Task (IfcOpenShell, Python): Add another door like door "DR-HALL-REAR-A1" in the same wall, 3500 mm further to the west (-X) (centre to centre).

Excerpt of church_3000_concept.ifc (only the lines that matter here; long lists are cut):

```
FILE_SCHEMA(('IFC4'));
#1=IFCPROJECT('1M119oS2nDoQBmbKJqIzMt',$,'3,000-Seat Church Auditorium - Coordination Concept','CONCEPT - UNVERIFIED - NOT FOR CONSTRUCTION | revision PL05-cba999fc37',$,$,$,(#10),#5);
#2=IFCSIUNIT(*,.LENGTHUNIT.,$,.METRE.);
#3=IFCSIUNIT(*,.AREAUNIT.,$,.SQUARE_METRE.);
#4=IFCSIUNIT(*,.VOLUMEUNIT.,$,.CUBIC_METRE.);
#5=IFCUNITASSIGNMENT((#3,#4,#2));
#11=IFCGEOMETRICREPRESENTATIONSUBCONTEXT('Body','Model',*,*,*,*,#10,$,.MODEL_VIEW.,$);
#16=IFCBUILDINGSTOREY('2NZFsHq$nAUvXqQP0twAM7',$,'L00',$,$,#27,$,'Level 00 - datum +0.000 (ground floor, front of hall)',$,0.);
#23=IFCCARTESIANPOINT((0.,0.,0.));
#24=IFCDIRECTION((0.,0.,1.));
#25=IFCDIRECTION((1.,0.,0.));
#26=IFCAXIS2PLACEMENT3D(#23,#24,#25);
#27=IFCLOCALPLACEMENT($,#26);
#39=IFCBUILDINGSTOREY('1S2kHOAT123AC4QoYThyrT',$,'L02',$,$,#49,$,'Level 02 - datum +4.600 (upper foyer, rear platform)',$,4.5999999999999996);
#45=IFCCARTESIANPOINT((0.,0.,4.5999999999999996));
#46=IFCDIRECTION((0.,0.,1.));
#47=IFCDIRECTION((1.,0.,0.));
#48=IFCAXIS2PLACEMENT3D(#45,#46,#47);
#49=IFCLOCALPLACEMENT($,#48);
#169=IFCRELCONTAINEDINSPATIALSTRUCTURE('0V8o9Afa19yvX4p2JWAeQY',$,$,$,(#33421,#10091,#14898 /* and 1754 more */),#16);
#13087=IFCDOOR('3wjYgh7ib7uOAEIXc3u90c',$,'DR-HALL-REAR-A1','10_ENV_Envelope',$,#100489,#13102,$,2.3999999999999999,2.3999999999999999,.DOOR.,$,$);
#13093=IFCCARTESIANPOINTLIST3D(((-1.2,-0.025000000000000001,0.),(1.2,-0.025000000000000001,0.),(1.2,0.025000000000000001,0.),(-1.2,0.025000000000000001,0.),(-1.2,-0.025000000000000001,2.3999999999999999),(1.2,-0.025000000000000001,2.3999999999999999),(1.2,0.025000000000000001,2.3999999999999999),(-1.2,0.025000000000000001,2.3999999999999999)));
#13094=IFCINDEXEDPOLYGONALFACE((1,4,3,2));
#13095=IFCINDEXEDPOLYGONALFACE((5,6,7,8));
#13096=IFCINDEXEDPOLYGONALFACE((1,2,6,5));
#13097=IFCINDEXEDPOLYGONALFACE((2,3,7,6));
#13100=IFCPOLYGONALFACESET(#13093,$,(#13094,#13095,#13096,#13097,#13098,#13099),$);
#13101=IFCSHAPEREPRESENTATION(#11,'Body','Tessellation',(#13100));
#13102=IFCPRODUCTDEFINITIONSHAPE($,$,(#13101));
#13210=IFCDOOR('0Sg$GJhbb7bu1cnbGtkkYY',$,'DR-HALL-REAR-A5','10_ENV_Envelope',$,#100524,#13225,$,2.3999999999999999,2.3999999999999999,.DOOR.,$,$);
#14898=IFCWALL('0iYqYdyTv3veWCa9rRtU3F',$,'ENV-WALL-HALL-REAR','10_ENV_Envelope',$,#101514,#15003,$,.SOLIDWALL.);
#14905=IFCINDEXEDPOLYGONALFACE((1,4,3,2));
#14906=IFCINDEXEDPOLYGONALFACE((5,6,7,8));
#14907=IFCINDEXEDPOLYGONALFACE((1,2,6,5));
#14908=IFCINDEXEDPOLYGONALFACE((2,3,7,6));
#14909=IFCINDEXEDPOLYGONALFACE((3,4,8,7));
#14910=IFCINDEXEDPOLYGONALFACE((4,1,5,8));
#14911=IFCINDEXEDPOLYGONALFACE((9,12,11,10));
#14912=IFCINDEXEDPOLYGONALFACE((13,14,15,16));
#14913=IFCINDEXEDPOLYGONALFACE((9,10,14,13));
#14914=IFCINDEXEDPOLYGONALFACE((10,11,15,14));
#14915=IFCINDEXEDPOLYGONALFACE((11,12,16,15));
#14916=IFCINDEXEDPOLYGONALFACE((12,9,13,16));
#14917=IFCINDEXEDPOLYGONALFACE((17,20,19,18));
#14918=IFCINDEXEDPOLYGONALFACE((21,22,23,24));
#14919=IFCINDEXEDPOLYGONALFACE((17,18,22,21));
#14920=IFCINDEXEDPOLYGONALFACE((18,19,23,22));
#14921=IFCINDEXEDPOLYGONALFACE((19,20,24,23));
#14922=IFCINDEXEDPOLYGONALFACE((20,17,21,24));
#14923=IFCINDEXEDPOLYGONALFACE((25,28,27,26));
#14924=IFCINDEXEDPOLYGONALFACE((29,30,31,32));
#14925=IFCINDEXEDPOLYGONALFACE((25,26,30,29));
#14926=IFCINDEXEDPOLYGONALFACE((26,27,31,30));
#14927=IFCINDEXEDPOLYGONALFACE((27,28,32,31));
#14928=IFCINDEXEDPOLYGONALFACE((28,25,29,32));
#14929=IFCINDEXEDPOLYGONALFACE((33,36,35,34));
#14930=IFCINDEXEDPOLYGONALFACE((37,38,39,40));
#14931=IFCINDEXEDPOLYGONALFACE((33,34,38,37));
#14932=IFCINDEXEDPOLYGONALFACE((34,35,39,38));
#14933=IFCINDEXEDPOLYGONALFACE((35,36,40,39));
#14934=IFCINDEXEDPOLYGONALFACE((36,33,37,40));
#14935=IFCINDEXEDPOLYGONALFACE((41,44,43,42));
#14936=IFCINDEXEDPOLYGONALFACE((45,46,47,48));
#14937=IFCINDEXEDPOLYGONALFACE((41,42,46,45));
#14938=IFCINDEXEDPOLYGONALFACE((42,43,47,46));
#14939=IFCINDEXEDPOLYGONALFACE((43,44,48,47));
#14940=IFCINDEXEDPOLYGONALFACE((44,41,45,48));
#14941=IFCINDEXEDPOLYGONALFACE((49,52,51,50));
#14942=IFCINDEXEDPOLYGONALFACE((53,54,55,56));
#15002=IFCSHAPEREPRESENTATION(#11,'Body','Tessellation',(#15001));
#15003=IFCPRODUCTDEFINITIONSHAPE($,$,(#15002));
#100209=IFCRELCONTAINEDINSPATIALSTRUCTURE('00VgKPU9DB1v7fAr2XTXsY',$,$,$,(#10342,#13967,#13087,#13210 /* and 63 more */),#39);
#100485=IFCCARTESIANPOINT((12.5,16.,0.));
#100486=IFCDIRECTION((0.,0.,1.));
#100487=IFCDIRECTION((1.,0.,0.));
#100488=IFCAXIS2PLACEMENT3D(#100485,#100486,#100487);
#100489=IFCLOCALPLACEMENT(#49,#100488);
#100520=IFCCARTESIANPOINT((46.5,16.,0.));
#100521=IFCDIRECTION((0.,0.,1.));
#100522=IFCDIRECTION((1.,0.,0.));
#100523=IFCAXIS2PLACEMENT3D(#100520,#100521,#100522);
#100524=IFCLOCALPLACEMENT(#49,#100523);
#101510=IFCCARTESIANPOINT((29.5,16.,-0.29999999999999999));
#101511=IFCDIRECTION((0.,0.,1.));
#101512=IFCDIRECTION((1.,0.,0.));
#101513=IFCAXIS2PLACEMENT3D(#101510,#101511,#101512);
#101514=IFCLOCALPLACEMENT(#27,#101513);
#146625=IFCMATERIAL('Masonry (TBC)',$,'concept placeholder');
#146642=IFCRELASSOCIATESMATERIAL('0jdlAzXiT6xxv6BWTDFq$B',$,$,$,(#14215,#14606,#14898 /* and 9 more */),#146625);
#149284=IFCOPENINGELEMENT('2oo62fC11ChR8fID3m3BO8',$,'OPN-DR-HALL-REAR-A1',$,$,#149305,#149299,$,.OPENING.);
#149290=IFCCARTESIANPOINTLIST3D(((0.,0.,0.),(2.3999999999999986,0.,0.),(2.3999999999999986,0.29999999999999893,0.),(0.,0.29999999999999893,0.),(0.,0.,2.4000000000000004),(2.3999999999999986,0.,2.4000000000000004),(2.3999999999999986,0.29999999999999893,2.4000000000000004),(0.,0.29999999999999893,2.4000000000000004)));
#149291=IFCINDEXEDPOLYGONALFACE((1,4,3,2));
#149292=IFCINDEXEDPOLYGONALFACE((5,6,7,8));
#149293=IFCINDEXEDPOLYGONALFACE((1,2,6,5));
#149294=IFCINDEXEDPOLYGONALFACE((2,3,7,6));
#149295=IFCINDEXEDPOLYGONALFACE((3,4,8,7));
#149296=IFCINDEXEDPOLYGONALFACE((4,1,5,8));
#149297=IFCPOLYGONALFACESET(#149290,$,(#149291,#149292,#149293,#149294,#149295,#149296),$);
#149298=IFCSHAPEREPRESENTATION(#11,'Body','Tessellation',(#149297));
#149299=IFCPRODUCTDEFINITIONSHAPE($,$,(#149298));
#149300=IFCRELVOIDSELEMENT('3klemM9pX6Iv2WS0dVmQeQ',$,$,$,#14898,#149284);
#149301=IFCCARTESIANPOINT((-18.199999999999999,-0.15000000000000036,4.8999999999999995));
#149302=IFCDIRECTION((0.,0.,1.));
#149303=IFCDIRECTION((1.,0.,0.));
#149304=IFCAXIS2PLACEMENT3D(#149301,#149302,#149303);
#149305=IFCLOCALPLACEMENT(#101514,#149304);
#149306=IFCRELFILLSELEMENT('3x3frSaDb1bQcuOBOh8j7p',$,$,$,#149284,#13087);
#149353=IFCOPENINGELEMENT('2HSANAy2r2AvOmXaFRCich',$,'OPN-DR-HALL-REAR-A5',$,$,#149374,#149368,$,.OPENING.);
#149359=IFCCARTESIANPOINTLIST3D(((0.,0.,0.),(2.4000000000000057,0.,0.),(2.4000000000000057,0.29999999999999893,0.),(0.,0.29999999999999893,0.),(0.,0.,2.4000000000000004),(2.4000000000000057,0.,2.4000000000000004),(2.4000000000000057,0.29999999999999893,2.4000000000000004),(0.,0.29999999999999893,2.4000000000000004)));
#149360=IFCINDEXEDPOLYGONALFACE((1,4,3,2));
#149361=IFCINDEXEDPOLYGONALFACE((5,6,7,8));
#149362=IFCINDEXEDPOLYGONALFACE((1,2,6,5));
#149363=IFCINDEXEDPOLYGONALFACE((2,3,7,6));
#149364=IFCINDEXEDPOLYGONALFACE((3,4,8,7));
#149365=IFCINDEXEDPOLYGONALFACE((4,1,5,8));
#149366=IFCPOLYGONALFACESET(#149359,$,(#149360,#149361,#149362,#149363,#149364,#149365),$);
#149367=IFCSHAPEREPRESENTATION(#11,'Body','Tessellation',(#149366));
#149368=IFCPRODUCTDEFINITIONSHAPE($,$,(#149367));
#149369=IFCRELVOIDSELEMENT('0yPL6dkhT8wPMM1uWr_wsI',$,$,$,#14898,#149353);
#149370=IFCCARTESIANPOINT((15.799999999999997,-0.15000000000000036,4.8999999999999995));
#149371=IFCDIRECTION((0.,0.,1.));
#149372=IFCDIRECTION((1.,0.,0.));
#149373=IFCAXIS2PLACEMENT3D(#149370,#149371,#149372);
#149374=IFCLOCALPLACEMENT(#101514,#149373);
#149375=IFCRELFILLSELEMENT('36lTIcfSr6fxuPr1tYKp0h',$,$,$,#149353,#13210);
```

```python
import ifcopenshell
import ifcopenshell.api.feature
import ifcopenshell.api.geometry
import ifcopenshell.api.root
import ifcopenshell.geom
import ifcopenshell.util.element
import ifcopenshell.util.placement
import ifcopenshell.util.shape
import ifcopenshell.util.unit

model = ifcopenshell.open("church_3000_concept.ifc")
unit_scale = ifcopenshell.util.unit.calculate_unit_scale(model)
settings = ifcopenshell.geom.settings()


def volume(element):
    """Net volume in cubic metres, openings subtracted."""
    shape = ifcopenshell.geom.create_shape(settings, element)
    return ifcopenshell.util.shape.get_volume(shape.geometry)


door = model.by_id(13087)
opening = door.FillsVoids[0].RelatingOpeningElement
wall = opening.VoidsElements[0].RelatingBuildingElement
before = volume(wall)
shift = ifcopenshell.util.placement.get_local_placement(wall.ObjectPlacement)[:3, 0] * -3.5 / unit_scale

# copy_class copies the void relationship, type, container and properties, but no geometry.
new_opening = ifcopenshell.api.root.copy_class(model, product=opening)
new_opening.Representation = ifcopenshell.util.element.copy_deep(
    model, opening.Representation, exclude=["IfcGeometricRepresentationContext", "IfcRepresentationMap"]
)
new_door = ifcopenshell.api.root.copy_class(model, product=door)
new_door.Representation = ifcopenshell.util.element.copy_deep(
    model, door.Representation, exclude=["IfcGeometricRepresentationContext", "IfcRepresentationMap"]
)
ifcopenshell.api.feature.add_filling(model, opening=new_opening, element=new_door)

for old, new in ((opening, new_opening), (door, new_door)):
    matrix = ifcopenshell.util.placement.get_local_placement(old.ObjectPlacement)
    matrix[:3, 3] += shift
    ifcopenshell.api.geometry.edit_object_placement(model, product=new, matrix=matrix, is_si=False)

after = volume(wall)

print(f"wall volume {before:.3f} -> {after:.3f} m3")

model.write("church_3000_concept_rev.ifc")
```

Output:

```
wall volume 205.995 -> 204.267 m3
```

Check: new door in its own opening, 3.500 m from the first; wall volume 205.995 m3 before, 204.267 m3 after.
